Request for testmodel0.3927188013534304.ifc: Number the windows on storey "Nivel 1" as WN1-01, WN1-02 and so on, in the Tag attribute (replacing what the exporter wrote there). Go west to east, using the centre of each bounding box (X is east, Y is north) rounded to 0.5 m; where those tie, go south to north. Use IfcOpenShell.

First a look at what the model holds.

```python
import ifcopenshell
import ifcopenshell.util.element
import ifcopenshell.util.placement

model = ifcopenshell.open("testmodel0.3927188013534304.ifc")
print(model.schema)
storey = next(s for s in model.by_type("IfcBuildingStorey") if s.Name == "Nivel 1")
windows = [e for e in ifcopenshell.util.element.get_decomposition(storey) if e.is_a("IfcWindow")]
for e in sorted(windows, key=lambda e: e.id()):
    origin = ifcopenshell.util.placement.get_local_placement(e.ObjectPlacement)[:3, 3]
    print(e.id(), e.Tag, e.Name, origin.round(2) + 0.0, sep=" | ")
```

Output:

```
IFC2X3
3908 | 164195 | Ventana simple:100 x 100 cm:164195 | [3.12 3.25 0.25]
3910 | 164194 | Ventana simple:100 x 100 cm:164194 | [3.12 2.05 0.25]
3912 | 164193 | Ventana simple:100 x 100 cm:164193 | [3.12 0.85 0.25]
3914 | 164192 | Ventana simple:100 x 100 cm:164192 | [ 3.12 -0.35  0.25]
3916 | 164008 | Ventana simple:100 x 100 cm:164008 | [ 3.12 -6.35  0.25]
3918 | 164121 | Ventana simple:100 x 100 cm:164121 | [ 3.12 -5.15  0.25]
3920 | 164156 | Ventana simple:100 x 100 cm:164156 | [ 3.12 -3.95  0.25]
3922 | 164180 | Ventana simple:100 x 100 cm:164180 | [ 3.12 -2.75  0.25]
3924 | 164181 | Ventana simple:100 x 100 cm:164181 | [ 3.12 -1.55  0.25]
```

```python
import ifcopenshell
import ifcopenshell.geom
import ifcopenshell.util.element
import ifcopenshell.util.shape

model = ifcopenshell.open("testmodel0.3927188013534304.ifc")
settings = ifcopenshell.geom.settings()
settings.set("use-world-coords", True)


def centre(element):
    shape = ifcopenshell.geom.create_shape(settings, element)
    return ifcopenshell.util.shape.get_bbox_centroid(shape.geometry)


storey = next(s for s in model.by_type("IfcBuildingStorey") if s.Name == "Nivel 1")
windows = [e for e in ifcopenshell.util.element.get_decomposition(storey) if e.is_a("IfcWindow")]

# Insertion points can sit at a corner or the storey origin, so sort by the geometry (in metres).
centres = {e: centre(e) for e in windows}
windows.sort(key=lambda e: (round(centres[e][0] / 0.5), centres[e][1]))

for i, e in enumerate(windows, start=1):
    number = f"WN1-{i:02d}"
    e.Tag = number
    print(e.id(), number)

model.write("testmodel0.3927188013534304_edited.ifc")
```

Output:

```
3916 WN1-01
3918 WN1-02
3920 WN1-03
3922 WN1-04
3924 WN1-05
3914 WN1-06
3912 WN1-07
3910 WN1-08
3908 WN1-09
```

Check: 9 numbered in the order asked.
